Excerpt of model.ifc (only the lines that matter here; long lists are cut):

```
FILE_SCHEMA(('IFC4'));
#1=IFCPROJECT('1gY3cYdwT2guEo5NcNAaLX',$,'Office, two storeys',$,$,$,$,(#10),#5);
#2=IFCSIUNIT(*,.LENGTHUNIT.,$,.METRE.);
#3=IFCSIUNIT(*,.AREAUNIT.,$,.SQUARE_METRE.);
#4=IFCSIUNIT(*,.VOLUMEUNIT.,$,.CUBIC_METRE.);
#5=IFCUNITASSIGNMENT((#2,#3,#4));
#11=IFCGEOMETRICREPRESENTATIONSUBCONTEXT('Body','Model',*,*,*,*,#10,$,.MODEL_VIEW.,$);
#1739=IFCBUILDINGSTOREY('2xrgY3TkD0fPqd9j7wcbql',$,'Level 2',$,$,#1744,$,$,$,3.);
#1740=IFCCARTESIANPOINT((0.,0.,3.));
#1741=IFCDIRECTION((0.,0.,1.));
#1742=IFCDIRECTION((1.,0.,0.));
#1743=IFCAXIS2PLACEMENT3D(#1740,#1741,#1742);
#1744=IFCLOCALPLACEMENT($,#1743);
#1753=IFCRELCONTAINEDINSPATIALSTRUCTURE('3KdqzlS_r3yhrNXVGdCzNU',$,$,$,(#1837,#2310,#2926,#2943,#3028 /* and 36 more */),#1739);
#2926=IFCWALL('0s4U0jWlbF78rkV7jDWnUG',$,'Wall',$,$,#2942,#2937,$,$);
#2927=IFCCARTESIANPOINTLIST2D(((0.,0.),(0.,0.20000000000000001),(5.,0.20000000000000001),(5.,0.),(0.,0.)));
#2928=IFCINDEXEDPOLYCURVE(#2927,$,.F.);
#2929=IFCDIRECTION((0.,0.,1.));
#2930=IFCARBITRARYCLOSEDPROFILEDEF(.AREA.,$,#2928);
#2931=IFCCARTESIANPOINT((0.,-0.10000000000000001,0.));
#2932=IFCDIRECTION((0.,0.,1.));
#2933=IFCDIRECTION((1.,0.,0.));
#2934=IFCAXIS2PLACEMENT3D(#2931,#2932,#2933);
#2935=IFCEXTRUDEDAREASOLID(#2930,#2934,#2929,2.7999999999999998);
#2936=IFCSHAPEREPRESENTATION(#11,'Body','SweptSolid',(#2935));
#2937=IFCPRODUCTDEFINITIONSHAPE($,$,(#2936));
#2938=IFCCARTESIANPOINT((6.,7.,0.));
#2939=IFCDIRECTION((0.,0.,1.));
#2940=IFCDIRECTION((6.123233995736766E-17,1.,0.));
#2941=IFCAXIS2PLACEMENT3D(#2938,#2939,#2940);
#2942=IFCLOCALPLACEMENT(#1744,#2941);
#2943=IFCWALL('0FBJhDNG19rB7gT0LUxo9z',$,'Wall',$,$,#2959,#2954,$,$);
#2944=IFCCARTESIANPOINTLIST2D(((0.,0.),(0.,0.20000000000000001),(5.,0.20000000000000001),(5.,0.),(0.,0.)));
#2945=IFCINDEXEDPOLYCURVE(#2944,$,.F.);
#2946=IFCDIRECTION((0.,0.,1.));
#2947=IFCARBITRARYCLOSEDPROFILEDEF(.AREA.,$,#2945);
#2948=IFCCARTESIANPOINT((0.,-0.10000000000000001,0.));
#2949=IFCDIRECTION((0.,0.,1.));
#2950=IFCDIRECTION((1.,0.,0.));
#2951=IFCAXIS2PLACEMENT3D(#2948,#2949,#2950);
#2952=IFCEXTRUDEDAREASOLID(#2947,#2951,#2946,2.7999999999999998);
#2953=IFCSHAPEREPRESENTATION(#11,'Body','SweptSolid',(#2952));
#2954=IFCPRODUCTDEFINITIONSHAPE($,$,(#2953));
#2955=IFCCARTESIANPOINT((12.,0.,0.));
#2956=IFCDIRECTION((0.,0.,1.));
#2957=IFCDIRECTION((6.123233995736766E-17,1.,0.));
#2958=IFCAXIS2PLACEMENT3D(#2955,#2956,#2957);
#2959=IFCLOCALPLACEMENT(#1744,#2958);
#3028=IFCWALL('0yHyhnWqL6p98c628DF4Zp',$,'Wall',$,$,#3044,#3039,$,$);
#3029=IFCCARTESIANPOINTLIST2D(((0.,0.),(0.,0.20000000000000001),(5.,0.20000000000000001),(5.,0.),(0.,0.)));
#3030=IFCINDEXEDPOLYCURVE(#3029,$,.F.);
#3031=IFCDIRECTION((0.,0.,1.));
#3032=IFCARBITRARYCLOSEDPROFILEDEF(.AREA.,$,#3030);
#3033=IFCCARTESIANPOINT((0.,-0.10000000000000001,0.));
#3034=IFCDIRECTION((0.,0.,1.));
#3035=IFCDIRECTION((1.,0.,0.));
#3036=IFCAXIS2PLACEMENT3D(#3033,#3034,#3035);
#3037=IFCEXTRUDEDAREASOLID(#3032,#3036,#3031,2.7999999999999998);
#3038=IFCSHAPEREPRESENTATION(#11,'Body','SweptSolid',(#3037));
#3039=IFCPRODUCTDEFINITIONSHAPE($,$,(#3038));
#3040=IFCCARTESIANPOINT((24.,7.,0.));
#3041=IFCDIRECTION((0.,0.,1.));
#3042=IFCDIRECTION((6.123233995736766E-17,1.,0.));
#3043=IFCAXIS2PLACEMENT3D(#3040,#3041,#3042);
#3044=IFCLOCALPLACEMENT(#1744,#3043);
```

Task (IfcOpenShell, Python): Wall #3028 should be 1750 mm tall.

```python
import ifcopenshell
import ifcopenshell.geom
import ifcopenshell.util.representation
import ifcopenshell.util.shape

model = ifcopenshell.open("model.ifc")
settings = ifcopenshell.geom.settings()


def volume(element):
    """Net volume in cubic metres, openings subtracted."""
    shape = ifcopenshell.geom.create_shape(settings, element)
    return ifcopenshell.util.shape.get_volume(shape.geometry)


wall = model.by_guid("0yHyhnWqL6p98c628DF4Zp")
before = volume(wall)

body = ifcopenshell.util.representation.get_representation(wall, "Model", "Body")
solid = body.Items[0]
old_height = solid.Depth
solid.Depth = 1.75
after = volume(wall)

print(f"height {old_height:g} -> {solid.Depth:g}, volume {before:.3f} -> {after:.3f} m3")

model.write("model_edited.ifc")
```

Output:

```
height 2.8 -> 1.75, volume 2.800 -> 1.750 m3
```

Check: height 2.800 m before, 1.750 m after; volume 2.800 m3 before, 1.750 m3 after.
